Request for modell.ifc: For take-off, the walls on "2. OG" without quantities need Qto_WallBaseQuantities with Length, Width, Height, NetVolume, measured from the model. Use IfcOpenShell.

First a look at what the model holds.

```python
import ifcopenshell
import ifcopenshell.util.element
import ifcopenshell.util.unit

model = ifcopenshell.open("modell.ifc")
print(model.schema)
for unit_type in ("LENGTHUNIT", "AREAUNIT", "VOLUMEUNIT"):
    print(unit_type, ifcopenshell.util.unit.calculate_unit_scale(model, unit_type))
storey = next(s for s in model.by_type("IfcBuildingStorey") if s.Name == "2. OG")
walls = [e for e in ifcopenshell.util.element.get_decomposition(storey) if e.is_a("IfcWall")]
for e in sorted(walls, key=lambda e: e.id()):
    print(e.id(), e.is_a(), e.Name, list(ifcopenshell.util.element.get_psets(e, qtos_only=True)), sep=" | ")
```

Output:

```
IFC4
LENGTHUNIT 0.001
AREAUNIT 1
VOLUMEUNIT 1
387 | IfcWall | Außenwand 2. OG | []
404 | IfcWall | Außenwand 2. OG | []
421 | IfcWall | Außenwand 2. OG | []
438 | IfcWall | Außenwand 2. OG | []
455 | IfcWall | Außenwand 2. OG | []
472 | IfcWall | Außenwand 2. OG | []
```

```python
import ifcopenshell
import ifcopenshell.api.pset
import ifcopenshell.geom
import ifcopenshell.util.element
import ifcopenshell.util.shape
import ifcopenshell.util.unit

model = ifcopenshell.open("modell.ifc")
unit_scale = ifcopenshell.util.unit.calculate_unit_scale(model)
volume_scale = ifcopenshell.util.unit.calculate_unit_scale(model, "VOLUMEUNIT")
settings = ifcopenshell.geom.settings()

storey = next(s for s in model.by_type("IfcBuildingStorey") if s.Name == "2. OG")
walls = [e for e in ifcopenshell.util.element.get_decomposition(storey) if e.is_a("IfcWall")]

for e in sorted(walls, key=lambda e: e.id()):
    if ifcopenshell.util.element.get_psets(e, qtos_only=True, should_inherit=False):
        continue
    # Geometry comes back in metres, in the element's own axes.
    shape = ifcopenshell.geom.create_shape(settings, e)
    values = {
        "Length": ifcopenshell.util.shape.get_x(shape.geometry) / unit_scale,
        "Width": ifcopenshell.util.shape.get_y(shape.geometry) / unit_scale,
        "Height": ifcopenshell.util.shape.get_z(shape.geometry) / unit_scale,
        "NetVolume": ifcopenshell.util.shape.get_volume(shape.geometry) / volume_scale,
    }
    qto = ifcopenshell.api.pset.add_qto(model, product=e, name="Qto_WallBaseQuantities")
    ifcopenshell.api.pset.edit_qto(model, qto=qto, properties=values)
    print(e.id(), {k: round(v, 3) for k, v in values.items()})

model.write("modell_updated.ifc")
```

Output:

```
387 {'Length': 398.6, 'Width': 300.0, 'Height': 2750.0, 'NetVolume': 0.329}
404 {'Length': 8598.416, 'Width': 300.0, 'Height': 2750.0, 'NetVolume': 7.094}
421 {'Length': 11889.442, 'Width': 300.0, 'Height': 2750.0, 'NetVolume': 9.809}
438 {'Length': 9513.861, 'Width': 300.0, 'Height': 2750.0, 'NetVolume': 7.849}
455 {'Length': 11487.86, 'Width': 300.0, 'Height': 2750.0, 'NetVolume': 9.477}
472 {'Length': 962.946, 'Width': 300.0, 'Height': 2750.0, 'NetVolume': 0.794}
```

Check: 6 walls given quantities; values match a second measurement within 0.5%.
